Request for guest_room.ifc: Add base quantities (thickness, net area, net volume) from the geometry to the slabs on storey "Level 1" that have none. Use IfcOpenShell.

First a look at what the model holds.

```python
import ifcopenshell
import ifcopenshell.util.element
import ifcopenshell.util.unit

model = ifcopenshell.open("guest_room.ifc")
print(model.schema)
for unit_type in ("LENGTHUNIT", "AREAUNIT", "VOLUMEUNIT"):
    print(unit_type, ifcopenshell.util.unit.calculate_unit_scale(model, unit_type))
storey = next(s for s in model.by_type("IfcBuildingStorey") if s.Name == "Level 1")
slabs = [e for e in ifcopenshell.util.element.get_decomposition(storey) if e.is_a("IfcSlab")]
for e in sorted(slabs, key=lambda e: e.id()):
    print(e.id(), e.is_a(), e.Name, list(ifcopenshell.util.element.get_psets(e, qtos_only=True)), sep=" | ")
```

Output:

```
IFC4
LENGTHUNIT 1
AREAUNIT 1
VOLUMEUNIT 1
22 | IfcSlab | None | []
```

```python
import ifcopenshell
import ifcopenshell.api.pset
import ifcopenshell.geom
import ifcopenshell.util.element
import ifcopenshell.util.shape
import ifcopenshell.util.unit

model = ifcopenshell.open("guest_room.ifc")
unit_scale = ifcopenshell.util.unit.calculate_unit_scale(model)
area_scale = ifcopenshell.util.unit.calculate_unit_scale(model, "AREAUNIT")
volume_scale = ifcopenshell.util.unit.calculate_unit_scale(model, "VOLUMEUNIT")
settings = ifcopenshell.geom.settings()

storey = next(s for s in model.by_type("IfcBuildingStorey") if s.Name == "Level 1")
slabs = [e for e in ifcopenshell.util.element.get_decomposition(storey) if e.is_a("IfcSlab")]

for e in sorted(slabs, key=lambda e: e.id()):
    if ifcopenshell.util.element.get_psets(e, qtos_only=True, should_inherit=False):
        continue
    # Geometry comes back in metres, in the element's own axes.
    shape = ifcopenshell.geom.create_shape(settings, e)
    values = {
        "Width": ifcopenshell.util.shape.get_z(shape.geometry) / unit_scale,
        "NetArea": ifcopenshell.util.shape.get_footprint_area(shape.geometry) / area_scale,
        "NetVolume": ifcopenshell.util.shape.get_volume(shape.geometry) / volume_scale,
    }
    qto = ifcopenshell.api.pset.add_qto(model, product=e, name="Qto_SlabBaseQuantities")
    ifcopenshell.api.pset.edit_qto(model, qto=qto, properties=values)
    print(e.id(), {k: round(v, 3) for k, v in values.items()})

model.write("guest_room_v2.ifc")
```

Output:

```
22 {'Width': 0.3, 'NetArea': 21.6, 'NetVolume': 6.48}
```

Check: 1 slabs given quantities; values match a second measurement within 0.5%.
